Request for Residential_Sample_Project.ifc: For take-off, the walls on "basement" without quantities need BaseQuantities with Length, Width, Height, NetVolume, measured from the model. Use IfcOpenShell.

First a look at what the model holds.

```python
import ifcopenshell
import ifcopenshell.util.element
import ifcopenshell.util.unit

model = ifcopenshell.open("Residential_Sample_Project.ifc")
print(model.schema)
for unit_type in ("LENGTHUNIT", "AREAUNIT", "VOLUMEUNIT"):
    print(unit_type, ifcopenshell.util.unit.calculate_unit_scale(model, unit_type))
storey = next(s for s in model.by_type("IfcBuildingStorey") if s.Name == "basement")
walls = [e for e in ifcopenshell.util.element.get_decomposition(storey) if e.is_a("IfcWall")]
for e in sorted(walls, key=lambda e: e.id()):
    print(e.id(), e.is_a(), e.Name, list(ifcopenshell.util.element.get_psets(e, qtos_only=True)), sep=" | ")
```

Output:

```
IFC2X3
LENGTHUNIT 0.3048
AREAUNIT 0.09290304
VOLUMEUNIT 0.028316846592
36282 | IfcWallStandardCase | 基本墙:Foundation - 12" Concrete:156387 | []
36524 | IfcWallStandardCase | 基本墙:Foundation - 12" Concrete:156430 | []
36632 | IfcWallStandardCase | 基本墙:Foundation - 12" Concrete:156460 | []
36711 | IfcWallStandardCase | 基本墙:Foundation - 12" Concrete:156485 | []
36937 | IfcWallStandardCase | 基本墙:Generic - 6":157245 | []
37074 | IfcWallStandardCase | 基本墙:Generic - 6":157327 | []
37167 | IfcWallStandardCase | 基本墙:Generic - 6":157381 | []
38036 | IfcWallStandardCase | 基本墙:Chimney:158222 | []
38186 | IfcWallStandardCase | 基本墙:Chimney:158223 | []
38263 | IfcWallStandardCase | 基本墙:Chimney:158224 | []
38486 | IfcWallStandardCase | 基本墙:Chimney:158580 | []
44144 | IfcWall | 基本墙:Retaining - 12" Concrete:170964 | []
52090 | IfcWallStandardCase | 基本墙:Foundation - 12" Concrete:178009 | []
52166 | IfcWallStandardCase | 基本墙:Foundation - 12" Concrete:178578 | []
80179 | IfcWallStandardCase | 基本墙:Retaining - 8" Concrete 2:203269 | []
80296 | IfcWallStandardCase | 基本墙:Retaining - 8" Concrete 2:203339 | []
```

```python
import ifcopenshell
import ifcopenshell.api.pset
import ifcopenshell.geom
import ifcopenshell.util.element
import ifcopenshell.util.shape
import ifcopenshell.util.unit

model = ifcopenshell.open("Residential_Sample_Project.ifc")
unit_scale = ifcopenshell.util.unit.calculate_unit_scale(model)
volume_scale = ifcopenshell.util.unit.calculate_unit_scale(model, "VOLUMEUNIT")
settings = ifcopenshell.geom.settings()

storey = next(s for s in model.by_type("IfcBuildingStorey") if s.Name == "basement")
walls = [e for e in ifcopenshell.util.element.get_decomposition(storey) if e.is_a("IfcWall")]

for e in sorted(walls, key=lambda e: e.id()):
    if ifcopenshell.util.element.get_psets(e, qtos_only=True, should_inherit=False):
        continue
    # Geometry comes back in metres, in the element's own axes.
    shape = ifcopenshell.geom.create_shape(settings, e)
    values = {
        "Length": ifcopenshell.util.shape.get_x(shape.geometry) / unit_scale,
        "Width": ifcopenshell.util.shape.get_y(shape.geometry) / unit_scale,
        "Height": ifcopenshell.util.shape.get_z(shape.geometry) / unit_scale,
        "NetVolume": ifcopenshell.util.shape.get_volume(shape.geometry) / volume_scale,
    }
    qto = ifcopenshell.api.pset.add_qto(model, product=e, name="BaseQuantities")
    ifcopenshell.api.pset.edit_qto(model, qto=qto, properties=values)
    print(e.id(), {k: round(v, 3) for k, v in values.items()})

model.write("Residential_Sample_Project_rev.ifc")
```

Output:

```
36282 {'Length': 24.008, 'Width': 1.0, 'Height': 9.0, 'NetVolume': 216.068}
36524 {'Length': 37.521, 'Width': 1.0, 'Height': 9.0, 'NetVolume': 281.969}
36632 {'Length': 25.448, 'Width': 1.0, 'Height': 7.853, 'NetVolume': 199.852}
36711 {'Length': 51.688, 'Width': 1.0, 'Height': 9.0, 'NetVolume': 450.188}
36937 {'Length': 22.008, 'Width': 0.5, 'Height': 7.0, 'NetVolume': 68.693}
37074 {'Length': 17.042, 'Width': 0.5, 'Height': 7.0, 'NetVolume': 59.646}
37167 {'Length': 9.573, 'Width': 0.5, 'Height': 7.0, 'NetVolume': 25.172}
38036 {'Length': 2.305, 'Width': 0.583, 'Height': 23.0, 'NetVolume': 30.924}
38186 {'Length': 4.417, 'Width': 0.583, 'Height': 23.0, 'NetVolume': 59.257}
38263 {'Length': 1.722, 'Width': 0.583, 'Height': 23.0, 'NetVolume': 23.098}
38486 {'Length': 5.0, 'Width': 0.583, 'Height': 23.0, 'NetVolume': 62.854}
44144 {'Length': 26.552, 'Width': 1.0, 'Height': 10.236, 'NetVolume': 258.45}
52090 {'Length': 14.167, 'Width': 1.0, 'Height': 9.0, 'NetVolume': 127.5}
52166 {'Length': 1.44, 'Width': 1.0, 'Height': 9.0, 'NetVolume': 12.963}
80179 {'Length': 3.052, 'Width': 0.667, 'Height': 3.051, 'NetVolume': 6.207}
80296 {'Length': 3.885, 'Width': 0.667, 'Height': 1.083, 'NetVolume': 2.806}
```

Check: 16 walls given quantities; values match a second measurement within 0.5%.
